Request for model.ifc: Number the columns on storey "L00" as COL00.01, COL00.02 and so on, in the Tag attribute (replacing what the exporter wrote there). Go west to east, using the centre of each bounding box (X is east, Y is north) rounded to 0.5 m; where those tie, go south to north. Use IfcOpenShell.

First a look at what the model holds.

```python
import ifcopenshell
import ifcopenshell.util.element
import ifcopenshell.util.placement

model = ifcopenshell.open("model.ifc")
print(model.schema)
storey = next(s for s in model.by_type("IfcBuildingStorey") if s.Name == "L00")
columns = [e for e in ifcopenshell.util.element.get_decomposition(storey) if e.is_a("IfcColumn")]
for e in sorted(columns, key=lambda e: e.id()):
    origin = ifcopenshell.util.placement.get_local_placement(e.ObjectPlacement)[:3, 3]
    print(e.id(), e.Tag, e.Name, origin.round(2) + 0.0, sep=" | ")
```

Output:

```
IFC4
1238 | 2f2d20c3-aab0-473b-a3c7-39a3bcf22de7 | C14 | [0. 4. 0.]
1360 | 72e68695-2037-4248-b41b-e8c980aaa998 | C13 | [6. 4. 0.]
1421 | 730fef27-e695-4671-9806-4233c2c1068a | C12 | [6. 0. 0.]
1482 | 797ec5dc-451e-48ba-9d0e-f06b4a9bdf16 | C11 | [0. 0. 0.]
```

```python
import ifcopenshell
import ifcopenshell.geom
import ifcopenshell.util.element
import ifcopenshell.util.shape

model = ifcopenshell.open("model.ifc")
settings = ifcopenshell.geom.settings()
settings.set("use-world-coords", True)


def centre(element):
    shape = ifcopenshell.geom.create_shape(settings, element)
    return ifcopenshell.util.shape.get_bbox_centroid(shape.geometry)


storey = next(s for s in model.by_type("IfcBuildingStorey") if s.Name == "L00")
columns = [e for e in ifcopenshell.util.element.get_decomposition(storey) if e.is_a("IfcColumn")]

# Insertion points can sit at a corner or the storey origin, so sort by the geometry (in metres).
centres = {e: centre(e) for e in columns}
columns.sort(key=lambda e: (round(centres[e][0] / 0.5), centres[e][1]))

for i, e in enumerate(columns, start=1):
    number = f"COL00.{i:02d}"
    e.Tag = number
    print(e.id(), number)

model.write("model_updated.ifc")
```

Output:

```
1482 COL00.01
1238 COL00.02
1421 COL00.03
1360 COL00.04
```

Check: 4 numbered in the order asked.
